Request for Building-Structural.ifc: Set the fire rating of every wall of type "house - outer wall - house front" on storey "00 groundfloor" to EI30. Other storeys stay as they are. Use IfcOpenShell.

First a look at what the model holds.

```python
import ifcopenshell
import ifcopenshell.util.element

model = ifcopenshell.open("Building-Structural.ifc")
print(model.schema)
storey = next(s for s in model.by_type("IfcBuildingStorey") if s.Name == "00 groundfloor")
walls = [e for e in ifcopenshell.util.element.get_decomposition(storey) if e.is_a("IfcWall")]
seen = {}
for e in walls:
    element_type = ifcopenshell.util.element.get_type(e)
    key = (element_type.Name if element_type != e and element_type else None, ifcopenshell.util.element.get_pset(e, "Pset_WallCommon", "FireRating"))
    seen[key] = seen.get(key, 0) + 1
for (name, value), count in sorted(seen.items(), key=str):
    print(count, "x", name, "|", value)
```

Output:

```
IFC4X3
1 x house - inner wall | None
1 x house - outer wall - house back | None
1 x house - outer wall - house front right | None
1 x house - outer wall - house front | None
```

```python
import ifcopenshell
import ifcopenshell.api.pset
import ifcopenshell.util.element

model = ifcopenshell.open("Building-Structural.ifc")

storey = next(s for s in model.by_type("IfcBuildingStorey") if s.Name == "00 groundfloor")
walls = [e for e in ifcopenshell.util.element.get_decomposition(storey) if e.is_a("IfcWall")]

count = 0
for e in walls:
    element_type = ifcopenshell.util.element.get_type(e)
    if element_type in (None, e) or element_type.Name != "house - outer wall - house front":
        continue
    # add_pset returns the element's existing set when there is one.
    pset = ifcopenshell.api.pset.add_pset(model, product=e, name="Pset_WallCommon")
    ifcopenshell.api.pset.edit_pset(model, pset=pset, properties={"FireRating": "EI30"})
    count += 1

print(count, "walls updated")

model.write("Building-Structural-out.ifc")
```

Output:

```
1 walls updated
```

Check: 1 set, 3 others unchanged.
